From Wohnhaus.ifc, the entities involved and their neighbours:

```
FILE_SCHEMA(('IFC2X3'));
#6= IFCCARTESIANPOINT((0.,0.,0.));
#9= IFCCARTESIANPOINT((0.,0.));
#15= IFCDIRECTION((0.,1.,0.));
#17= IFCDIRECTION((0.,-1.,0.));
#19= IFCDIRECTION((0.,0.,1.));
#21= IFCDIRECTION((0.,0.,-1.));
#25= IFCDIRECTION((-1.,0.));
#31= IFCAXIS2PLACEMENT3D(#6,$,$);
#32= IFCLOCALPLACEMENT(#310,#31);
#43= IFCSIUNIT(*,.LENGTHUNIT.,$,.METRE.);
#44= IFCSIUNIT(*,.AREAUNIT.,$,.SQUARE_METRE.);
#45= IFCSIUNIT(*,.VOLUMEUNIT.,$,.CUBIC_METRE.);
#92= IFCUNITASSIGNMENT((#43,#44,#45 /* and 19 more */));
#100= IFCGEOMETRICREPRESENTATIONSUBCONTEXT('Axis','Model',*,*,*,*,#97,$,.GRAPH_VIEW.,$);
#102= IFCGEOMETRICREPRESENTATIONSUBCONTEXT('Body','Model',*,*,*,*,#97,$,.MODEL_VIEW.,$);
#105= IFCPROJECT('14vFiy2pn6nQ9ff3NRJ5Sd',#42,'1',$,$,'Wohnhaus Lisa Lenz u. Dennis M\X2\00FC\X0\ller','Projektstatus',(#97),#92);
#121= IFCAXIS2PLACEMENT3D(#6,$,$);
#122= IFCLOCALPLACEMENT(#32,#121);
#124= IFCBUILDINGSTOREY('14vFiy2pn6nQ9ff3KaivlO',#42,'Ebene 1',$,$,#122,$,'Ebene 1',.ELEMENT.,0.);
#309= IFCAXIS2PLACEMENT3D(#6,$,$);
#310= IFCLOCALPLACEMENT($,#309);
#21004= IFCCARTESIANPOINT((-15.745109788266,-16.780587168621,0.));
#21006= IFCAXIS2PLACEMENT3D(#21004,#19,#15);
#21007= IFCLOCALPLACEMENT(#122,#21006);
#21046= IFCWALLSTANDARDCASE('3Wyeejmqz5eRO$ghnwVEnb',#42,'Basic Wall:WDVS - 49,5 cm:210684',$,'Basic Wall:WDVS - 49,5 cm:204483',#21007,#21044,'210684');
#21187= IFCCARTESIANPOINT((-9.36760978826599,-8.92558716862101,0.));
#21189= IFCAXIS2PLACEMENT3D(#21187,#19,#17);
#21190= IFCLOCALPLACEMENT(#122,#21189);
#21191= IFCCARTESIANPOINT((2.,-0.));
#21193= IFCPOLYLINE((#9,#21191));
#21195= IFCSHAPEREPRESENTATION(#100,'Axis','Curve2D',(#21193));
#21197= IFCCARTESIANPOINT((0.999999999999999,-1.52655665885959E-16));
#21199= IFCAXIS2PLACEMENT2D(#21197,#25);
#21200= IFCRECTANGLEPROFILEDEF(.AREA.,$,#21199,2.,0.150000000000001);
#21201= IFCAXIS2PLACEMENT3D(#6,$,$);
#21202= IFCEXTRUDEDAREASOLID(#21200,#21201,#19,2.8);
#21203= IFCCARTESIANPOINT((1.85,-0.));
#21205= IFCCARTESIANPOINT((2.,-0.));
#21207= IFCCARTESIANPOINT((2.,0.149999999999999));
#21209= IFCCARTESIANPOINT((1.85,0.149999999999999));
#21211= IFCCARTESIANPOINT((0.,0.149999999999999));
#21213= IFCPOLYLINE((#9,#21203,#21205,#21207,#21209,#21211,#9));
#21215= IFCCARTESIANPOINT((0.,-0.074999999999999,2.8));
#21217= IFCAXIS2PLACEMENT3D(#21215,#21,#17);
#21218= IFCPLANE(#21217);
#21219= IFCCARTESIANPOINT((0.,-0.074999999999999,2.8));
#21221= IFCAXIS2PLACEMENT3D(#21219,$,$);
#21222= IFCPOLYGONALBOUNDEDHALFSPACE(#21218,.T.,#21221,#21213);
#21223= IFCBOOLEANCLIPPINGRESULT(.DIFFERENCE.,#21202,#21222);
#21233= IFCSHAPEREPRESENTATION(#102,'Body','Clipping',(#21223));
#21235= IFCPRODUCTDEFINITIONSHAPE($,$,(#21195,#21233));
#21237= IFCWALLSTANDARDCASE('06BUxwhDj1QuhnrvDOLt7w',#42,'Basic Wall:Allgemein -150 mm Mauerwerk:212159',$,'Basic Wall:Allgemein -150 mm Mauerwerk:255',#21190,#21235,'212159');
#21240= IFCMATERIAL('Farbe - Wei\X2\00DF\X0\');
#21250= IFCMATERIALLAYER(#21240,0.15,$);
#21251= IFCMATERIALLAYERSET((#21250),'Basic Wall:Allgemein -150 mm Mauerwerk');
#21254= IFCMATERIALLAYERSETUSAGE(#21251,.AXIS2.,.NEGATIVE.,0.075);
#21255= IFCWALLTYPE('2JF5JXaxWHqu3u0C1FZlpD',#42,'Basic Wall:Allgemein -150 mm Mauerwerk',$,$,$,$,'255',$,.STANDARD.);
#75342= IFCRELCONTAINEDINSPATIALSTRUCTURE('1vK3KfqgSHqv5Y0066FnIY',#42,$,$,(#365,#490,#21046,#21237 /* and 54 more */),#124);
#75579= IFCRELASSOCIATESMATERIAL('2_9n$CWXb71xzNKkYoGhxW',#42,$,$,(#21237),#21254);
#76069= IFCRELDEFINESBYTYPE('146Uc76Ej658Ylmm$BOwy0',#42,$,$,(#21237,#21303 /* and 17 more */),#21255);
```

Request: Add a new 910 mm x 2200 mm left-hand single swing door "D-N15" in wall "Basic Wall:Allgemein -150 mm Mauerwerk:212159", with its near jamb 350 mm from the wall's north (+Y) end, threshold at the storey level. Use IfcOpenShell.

```python
import numpy as np
import ifcopenshell
import ifcopenshell.api.feature
import ifcopenshell.api.geometry
import ifcopenshell.api.root
import ifcopenshell.api.spatial
import ifcopenshell.api.type
import ifcopenshell.geom
import ifcopenshell.util.element
import ifcopenshell.util.placement
import ifcopenshell.util.representation
import ifcopenshell.util.shape
import ifcopenshell.util.unit

model = ifcopenshell.open("Wohnhaus.ifc")
unit_scale = ifcopenshell.util.unit.calculate_unit_scale(model)
settings = ifcopenshell.geom.settings()


def volume(element):
    """Net volume in cubic metres, openings subtracted."""
    shape = ifcopenshell.geom.create_shape(settings, element)
    return ifcopenshell.util.shape.get_volume(shape.geometry)


wall = model.by_guid("06BUxwhDj1QuhnrvDOLt7w")
storey = ifcopenshell.util.element.get_container(wall, ifc_class="IfcBuildingStorey")
context = ifcopenshell.util.representation.get_context(model, "Model", "Body", "MODEL_VIEW")
before = volume(wall)

width, height, from_end, sill = 0.91, 2.2, 0.35, 0.0  # metres

# The wall runs along its own X axis, and the end named is its -X end.
wall_shape = ifcopenshell.geom.create_shape(settings, wall)
x, y, z = ifcopenshell.util.shape.get_vertices(wall_shape.geometry).T
start = x.min() + from_end
face, thickness = float(y.min()), float(y.max() - y.min())
wall_matrix = ifcopenshell.util.placement.get_local_placement(wall.ObjectPlacement)
level = ifcopenshell.util.placement.get_local_placement(storey.ObjectPlacement)[2, 3]


def in_wall(x, y):
    """Placement at x, y metres in the wall's axes, at sill height."""
    matrix = wall_matrix.copy()
    matrix[:, 3] = wall_matrix @ np.array([x / unit_scale, y / unit_scale, 0.0, 1.0])
    matrix[2, 3] = level + sill / unit_scale
    return matrix


# Opening: a box that overshoots both wall faces by 50 mm.
opening = ifcopenshell.api.root.create_entity(model, ifc_class="IfcOpeningElement")
box = ifcopenshell.api.geometry.add_wall_representation(
    model, context=context, length=width, height=height, thickness=thickness + 0.1
)
ifcopenshell.api.geometry.assign_representation(model, product=opening, representation=box)
ifcopenshell.api.geometry.edit_object_placement(model, product=opening, matrix=in_wall(start, face - 0.05), is_si=False)
ifcopenshell.api.feature.add_feature(model, feature=opening, element=wall)

door = ifcopenshell.api.root.create_entity(model, ifc_class="IfcDoor", name="D-N15")
door.OverallWidth, door.OverallHeight = width / unit_scale, height / unit_scale
body = ifcopenshell.api.geometry.add_door_representation(
    model,
    context=context,
    overall_width=door.OverallWidth,
    overall_height=door.OverallHeight,
    operation_type="SINGLE_SWING_LEFT",
    lining_properties={"LiningDepth": thickness / unit_scale, "ThresholdDepth": thickness / unit_scale},
)
ifcopenshell.api.geometry.assign_representation(model, product=door, representation=body)
ifcopenshell.api.spatial.assign_container(model, products=[door], relating_structure=storey)
fills = ifcopenshell.api.feature.add_filling(model, opening=opening, element=door)
fills.OwnerHistory = door.OwnerHistory  # required in IFC2X3

# IFC2X3 keeps the operation on the door style.
style = ifcopenshell.api.root.create_entity(model, ifc_class="IfcDoorStyle", name="D-N15")
style.OperationType, style.ConstructionType = "SINGLE_SWING_LEFT", "NOTDEFINED"
style.ParameterTakesPrecedence = style.Sizeable = False
ifcopenshell.api.type.assign_type(model, related_objects=[door], relating_type=style)

# The lining spans the wall, so the door starts at the wall face.
ifcopenshell.api.geometry.edit_object_placement(model, product=door, matrix=in_wall(start, face), is_si=False)

after = volume(wall)

print(f"wall volume {before:.3f} -> {after:.3f} m3")

model.write("Wohnhaus_v2.ifc")
```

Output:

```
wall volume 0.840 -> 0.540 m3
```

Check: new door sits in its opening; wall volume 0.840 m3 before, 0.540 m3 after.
